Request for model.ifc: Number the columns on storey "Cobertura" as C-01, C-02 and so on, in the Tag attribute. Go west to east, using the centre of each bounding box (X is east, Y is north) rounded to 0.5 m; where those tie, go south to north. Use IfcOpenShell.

First a look at what the model holds.

```python
import ifcopenshell
import ifcopenshell.util.element
import ifcopenshell.util.placement

model = ifcopenshell.open("model.ifc")
print(model.schema)
storey = next(s for s in model.by_type("IfcBuildingStorey") if s.Name == "Cobertura")
columns = [e for e in ifcopenshell.util.element.get_decomposition(storey) if e.is_a("IfcColumn")]
for e in sorted(columns, key=lambda e: e.id()):
    origin = ifcopenshell.util.placement.get_local_placement(e.ObjectPlacement)[:3, 3]
    print(e.id(), e.Tag, e.Name, origin.round(2) + 0.0, sep=" | ")
```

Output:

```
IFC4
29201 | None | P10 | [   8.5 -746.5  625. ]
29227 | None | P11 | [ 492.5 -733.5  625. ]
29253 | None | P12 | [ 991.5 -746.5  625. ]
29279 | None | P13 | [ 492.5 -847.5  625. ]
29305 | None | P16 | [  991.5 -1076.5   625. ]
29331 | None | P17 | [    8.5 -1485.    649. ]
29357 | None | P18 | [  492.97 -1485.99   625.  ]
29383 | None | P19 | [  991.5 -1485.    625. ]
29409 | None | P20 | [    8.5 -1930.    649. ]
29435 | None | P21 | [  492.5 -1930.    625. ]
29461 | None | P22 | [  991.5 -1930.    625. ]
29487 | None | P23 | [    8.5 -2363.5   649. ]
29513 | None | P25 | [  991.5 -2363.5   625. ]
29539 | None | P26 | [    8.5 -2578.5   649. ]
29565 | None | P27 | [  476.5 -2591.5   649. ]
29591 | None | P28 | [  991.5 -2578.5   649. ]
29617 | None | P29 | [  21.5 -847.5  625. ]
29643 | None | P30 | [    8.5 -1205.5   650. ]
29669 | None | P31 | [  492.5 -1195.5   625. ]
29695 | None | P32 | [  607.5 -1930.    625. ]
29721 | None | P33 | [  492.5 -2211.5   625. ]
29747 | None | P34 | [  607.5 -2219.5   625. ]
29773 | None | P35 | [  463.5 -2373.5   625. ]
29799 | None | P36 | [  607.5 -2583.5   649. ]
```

```python
import ifcopenshell
import ifcopenshell.geom
import ifcopenshell.util.element
import ifcopenshell.util.shape

model = ifcopenshell.open("model.ifc")
settings = ifcopenshell.geom.settings()
settings.set("use-world-coords", True)


def centre(element):
    shape = ifcopenshell.geom.create_shape(settings, element)
    return ifcopenshell.util.shape.get_bbox_centroid(shape.geometry)


storey = next(s for s in model.by_type("IfcBuildingStorey") if s.Name == "Cobertura")
columns = [e for e in ifcopenshell.util.element.get_decomposition(storey) if e.is_a("IfcColumn")]

# Insertion points can sit at a corner or the storey origin, so sort by the geometry (in metres).
centres = {e: centre(e) for e in columns}
columns.sort(key=lambda e: (round(centres[e][0] / 0.5), centres[e][1]))

for i, e in enumerate(columns, start=1):
    number = f"C-{i:02d}"
    e.Tag = number
    print(e.id(), number)

model.write("model_v2.ifc")
```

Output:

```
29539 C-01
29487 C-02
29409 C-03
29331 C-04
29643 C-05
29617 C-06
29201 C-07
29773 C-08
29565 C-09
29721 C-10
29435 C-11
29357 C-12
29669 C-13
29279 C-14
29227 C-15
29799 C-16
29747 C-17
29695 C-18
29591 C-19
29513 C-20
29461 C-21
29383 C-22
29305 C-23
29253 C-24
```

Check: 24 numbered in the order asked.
